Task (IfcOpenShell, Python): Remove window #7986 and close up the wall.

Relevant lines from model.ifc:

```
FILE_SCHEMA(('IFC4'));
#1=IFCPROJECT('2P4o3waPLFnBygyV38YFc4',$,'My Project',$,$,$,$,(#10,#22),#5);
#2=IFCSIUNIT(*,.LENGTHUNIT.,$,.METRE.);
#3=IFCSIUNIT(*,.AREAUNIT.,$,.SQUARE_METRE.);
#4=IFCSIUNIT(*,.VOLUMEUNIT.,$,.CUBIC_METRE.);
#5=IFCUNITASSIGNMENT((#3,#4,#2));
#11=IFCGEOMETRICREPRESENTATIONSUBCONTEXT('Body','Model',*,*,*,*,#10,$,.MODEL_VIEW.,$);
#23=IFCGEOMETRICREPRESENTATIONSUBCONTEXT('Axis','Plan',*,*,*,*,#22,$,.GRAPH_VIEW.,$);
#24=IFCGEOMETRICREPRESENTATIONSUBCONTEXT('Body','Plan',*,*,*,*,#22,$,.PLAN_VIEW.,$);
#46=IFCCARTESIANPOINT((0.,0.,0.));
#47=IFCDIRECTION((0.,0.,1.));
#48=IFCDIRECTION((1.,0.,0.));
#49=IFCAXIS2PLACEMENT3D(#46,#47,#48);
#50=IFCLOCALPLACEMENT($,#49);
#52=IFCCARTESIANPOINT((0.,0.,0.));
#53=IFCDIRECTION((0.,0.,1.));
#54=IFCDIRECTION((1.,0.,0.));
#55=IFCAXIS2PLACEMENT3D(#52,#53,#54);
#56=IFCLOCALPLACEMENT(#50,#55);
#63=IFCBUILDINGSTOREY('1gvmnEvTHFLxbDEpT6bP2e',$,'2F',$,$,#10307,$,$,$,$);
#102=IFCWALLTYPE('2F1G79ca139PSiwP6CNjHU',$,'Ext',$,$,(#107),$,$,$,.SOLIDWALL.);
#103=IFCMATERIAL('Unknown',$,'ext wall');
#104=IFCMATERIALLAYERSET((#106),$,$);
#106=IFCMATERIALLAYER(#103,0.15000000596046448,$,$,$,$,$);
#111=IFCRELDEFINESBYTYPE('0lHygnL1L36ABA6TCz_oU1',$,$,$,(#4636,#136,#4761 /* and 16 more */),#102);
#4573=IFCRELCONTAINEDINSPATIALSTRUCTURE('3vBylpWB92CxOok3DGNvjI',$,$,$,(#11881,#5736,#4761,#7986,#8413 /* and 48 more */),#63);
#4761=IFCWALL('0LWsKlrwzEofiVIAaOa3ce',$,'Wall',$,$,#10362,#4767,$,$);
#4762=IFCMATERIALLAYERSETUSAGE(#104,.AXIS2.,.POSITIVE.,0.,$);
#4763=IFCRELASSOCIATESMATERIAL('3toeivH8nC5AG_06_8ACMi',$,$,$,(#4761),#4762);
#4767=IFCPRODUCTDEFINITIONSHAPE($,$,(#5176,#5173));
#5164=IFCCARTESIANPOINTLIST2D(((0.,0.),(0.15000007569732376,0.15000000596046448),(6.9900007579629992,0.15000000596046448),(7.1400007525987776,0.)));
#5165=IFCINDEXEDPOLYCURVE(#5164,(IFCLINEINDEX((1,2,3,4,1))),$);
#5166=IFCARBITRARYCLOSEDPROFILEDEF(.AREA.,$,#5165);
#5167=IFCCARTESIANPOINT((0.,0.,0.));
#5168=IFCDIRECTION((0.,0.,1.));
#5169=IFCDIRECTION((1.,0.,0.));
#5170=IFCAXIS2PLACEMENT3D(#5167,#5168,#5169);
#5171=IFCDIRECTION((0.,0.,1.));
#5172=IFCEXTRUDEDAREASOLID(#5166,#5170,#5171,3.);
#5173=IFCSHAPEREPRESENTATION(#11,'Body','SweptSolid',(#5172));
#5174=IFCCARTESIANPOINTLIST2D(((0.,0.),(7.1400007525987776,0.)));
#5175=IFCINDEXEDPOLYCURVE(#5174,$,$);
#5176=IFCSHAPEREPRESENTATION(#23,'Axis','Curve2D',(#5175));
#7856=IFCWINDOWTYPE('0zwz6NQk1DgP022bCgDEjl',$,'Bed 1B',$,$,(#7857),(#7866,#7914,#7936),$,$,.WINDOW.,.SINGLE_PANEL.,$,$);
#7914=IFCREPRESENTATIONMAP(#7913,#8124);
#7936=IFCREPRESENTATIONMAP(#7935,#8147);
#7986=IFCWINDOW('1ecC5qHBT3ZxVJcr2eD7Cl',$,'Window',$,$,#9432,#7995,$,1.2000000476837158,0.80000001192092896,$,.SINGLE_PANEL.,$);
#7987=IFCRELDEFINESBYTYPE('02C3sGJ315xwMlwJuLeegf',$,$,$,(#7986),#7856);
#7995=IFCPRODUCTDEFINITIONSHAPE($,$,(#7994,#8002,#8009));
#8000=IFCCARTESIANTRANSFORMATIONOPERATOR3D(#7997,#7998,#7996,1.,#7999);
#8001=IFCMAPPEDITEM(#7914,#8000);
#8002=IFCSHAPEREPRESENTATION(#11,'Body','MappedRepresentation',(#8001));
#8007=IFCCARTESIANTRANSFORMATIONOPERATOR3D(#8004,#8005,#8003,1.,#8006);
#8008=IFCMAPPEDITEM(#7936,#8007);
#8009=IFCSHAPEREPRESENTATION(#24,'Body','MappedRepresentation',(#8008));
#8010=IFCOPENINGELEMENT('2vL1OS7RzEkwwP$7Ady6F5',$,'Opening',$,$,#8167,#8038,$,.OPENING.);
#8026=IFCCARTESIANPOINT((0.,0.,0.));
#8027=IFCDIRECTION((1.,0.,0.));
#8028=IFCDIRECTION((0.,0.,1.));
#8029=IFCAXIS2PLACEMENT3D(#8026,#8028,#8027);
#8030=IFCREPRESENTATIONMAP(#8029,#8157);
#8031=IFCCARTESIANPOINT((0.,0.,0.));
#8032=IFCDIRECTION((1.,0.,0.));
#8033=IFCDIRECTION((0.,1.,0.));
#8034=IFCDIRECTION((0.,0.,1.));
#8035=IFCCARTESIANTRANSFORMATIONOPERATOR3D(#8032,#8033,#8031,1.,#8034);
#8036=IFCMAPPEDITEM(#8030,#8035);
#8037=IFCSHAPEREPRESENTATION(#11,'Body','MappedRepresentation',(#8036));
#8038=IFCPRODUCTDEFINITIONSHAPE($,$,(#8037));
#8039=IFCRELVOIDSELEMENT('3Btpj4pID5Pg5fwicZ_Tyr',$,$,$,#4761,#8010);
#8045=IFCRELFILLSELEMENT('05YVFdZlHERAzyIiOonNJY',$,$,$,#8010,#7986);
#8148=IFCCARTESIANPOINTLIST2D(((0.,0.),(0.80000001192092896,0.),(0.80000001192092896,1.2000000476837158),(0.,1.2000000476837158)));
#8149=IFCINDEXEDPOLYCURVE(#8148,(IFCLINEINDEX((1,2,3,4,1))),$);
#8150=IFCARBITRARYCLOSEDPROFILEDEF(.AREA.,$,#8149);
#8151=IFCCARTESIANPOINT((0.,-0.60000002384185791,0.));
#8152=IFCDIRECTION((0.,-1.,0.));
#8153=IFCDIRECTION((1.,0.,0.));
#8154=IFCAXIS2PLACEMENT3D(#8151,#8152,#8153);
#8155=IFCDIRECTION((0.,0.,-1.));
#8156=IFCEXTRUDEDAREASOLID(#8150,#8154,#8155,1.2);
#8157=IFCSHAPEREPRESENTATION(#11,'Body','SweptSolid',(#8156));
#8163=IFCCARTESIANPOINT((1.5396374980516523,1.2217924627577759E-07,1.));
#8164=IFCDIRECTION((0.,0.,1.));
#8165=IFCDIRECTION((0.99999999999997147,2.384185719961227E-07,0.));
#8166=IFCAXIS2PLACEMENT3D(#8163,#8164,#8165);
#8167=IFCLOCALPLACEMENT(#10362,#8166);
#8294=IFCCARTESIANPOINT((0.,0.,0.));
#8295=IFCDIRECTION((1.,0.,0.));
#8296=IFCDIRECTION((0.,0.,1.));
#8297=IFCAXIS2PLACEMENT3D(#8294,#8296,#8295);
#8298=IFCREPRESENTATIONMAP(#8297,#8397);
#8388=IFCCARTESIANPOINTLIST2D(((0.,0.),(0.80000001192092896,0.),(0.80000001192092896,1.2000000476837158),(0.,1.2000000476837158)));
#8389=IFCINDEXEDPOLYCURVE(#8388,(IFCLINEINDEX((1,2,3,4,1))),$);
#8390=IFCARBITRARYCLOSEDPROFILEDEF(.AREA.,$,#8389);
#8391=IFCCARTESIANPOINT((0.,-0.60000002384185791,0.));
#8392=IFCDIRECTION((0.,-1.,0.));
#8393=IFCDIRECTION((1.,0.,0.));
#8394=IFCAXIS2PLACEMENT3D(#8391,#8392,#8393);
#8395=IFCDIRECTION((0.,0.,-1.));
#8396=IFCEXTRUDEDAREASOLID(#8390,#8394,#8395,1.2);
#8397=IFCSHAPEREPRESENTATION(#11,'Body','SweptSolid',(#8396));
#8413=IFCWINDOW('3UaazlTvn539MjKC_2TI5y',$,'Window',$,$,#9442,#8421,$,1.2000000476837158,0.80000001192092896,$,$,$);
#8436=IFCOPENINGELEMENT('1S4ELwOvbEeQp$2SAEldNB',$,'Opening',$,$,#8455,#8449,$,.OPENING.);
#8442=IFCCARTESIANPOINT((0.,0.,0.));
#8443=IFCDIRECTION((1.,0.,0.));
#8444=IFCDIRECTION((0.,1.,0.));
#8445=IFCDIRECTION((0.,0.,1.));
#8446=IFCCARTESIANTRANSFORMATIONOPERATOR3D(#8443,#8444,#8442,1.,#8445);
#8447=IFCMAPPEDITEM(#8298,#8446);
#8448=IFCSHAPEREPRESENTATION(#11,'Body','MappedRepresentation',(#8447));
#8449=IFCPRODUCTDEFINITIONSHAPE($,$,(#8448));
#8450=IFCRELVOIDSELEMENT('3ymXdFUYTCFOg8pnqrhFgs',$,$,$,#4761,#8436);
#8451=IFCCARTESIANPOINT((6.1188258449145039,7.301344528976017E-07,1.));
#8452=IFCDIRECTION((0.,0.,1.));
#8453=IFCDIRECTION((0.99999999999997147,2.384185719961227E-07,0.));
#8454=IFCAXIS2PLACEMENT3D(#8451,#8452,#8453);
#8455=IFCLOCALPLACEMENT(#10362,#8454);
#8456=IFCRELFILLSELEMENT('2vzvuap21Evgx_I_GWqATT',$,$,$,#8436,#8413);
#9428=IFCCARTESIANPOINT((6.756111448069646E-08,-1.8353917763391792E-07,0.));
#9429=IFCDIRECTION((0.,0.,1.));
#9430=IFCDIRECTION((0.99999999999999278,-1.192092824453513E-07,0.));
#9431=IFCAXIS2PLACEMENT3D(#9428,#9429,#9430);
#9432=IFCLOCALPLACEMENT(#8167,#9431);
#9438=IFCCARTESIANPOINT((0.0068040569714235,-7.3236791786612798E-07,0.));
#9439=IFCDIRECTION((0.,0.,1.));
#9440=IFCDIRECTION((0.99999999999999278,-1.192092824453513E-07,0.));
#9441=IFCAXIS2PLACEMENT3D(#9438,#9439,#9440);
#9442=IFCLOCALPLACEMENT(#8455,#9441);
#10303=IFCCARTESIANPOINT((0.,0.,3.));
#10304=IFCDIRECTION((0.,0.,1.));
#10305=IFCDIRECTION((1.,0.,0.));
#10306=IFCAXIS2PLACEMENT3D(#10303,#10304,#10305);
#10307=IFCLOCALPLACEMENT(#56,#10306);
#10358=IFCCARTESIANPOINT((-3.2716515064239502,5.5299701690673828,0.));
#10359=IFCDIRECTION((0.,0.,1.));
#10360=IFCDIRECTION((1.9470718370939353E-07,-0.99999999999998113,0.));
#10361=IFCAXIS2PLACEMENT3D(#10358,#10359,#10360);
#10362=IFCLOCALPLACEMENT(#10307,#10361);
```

```python
import ifcopenshell
import ifcopenshell.api.feature
import ifcopenshell.api.root
import ifcopenshell.geom
import ifcopenshell.util.shape

model = ifcopenshell.open("model.ifc")
settings = ifcopenshell.geom.settings()


def volume(element):
    """Net volume in cubic metres, openings subtracted."""
    shape = ifcopenshell.geom.create_shape(settings, element)
    return ifcopenshell.util.shape.get_volume(shape.geometry)


window = model.by_id(7986)
opening = window.FillsVoids[0].RelatingOpeningElement
wall = opening.VoidsElements[0].RelatingBuildingElement
before = volume(wall)

ifcopenshell.api.root.remove_product(model, product=window)
ifcopenshell.api.feature.remove_feature(model, feature=opening)

after = volume(wall)

print(f"wall volume {before:.3f} -> {after:.3f} m3")

model.write("model_edited.ifc")
```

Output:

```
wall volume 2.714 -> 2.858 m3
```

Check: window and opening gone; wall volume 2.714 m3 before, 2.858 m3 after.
